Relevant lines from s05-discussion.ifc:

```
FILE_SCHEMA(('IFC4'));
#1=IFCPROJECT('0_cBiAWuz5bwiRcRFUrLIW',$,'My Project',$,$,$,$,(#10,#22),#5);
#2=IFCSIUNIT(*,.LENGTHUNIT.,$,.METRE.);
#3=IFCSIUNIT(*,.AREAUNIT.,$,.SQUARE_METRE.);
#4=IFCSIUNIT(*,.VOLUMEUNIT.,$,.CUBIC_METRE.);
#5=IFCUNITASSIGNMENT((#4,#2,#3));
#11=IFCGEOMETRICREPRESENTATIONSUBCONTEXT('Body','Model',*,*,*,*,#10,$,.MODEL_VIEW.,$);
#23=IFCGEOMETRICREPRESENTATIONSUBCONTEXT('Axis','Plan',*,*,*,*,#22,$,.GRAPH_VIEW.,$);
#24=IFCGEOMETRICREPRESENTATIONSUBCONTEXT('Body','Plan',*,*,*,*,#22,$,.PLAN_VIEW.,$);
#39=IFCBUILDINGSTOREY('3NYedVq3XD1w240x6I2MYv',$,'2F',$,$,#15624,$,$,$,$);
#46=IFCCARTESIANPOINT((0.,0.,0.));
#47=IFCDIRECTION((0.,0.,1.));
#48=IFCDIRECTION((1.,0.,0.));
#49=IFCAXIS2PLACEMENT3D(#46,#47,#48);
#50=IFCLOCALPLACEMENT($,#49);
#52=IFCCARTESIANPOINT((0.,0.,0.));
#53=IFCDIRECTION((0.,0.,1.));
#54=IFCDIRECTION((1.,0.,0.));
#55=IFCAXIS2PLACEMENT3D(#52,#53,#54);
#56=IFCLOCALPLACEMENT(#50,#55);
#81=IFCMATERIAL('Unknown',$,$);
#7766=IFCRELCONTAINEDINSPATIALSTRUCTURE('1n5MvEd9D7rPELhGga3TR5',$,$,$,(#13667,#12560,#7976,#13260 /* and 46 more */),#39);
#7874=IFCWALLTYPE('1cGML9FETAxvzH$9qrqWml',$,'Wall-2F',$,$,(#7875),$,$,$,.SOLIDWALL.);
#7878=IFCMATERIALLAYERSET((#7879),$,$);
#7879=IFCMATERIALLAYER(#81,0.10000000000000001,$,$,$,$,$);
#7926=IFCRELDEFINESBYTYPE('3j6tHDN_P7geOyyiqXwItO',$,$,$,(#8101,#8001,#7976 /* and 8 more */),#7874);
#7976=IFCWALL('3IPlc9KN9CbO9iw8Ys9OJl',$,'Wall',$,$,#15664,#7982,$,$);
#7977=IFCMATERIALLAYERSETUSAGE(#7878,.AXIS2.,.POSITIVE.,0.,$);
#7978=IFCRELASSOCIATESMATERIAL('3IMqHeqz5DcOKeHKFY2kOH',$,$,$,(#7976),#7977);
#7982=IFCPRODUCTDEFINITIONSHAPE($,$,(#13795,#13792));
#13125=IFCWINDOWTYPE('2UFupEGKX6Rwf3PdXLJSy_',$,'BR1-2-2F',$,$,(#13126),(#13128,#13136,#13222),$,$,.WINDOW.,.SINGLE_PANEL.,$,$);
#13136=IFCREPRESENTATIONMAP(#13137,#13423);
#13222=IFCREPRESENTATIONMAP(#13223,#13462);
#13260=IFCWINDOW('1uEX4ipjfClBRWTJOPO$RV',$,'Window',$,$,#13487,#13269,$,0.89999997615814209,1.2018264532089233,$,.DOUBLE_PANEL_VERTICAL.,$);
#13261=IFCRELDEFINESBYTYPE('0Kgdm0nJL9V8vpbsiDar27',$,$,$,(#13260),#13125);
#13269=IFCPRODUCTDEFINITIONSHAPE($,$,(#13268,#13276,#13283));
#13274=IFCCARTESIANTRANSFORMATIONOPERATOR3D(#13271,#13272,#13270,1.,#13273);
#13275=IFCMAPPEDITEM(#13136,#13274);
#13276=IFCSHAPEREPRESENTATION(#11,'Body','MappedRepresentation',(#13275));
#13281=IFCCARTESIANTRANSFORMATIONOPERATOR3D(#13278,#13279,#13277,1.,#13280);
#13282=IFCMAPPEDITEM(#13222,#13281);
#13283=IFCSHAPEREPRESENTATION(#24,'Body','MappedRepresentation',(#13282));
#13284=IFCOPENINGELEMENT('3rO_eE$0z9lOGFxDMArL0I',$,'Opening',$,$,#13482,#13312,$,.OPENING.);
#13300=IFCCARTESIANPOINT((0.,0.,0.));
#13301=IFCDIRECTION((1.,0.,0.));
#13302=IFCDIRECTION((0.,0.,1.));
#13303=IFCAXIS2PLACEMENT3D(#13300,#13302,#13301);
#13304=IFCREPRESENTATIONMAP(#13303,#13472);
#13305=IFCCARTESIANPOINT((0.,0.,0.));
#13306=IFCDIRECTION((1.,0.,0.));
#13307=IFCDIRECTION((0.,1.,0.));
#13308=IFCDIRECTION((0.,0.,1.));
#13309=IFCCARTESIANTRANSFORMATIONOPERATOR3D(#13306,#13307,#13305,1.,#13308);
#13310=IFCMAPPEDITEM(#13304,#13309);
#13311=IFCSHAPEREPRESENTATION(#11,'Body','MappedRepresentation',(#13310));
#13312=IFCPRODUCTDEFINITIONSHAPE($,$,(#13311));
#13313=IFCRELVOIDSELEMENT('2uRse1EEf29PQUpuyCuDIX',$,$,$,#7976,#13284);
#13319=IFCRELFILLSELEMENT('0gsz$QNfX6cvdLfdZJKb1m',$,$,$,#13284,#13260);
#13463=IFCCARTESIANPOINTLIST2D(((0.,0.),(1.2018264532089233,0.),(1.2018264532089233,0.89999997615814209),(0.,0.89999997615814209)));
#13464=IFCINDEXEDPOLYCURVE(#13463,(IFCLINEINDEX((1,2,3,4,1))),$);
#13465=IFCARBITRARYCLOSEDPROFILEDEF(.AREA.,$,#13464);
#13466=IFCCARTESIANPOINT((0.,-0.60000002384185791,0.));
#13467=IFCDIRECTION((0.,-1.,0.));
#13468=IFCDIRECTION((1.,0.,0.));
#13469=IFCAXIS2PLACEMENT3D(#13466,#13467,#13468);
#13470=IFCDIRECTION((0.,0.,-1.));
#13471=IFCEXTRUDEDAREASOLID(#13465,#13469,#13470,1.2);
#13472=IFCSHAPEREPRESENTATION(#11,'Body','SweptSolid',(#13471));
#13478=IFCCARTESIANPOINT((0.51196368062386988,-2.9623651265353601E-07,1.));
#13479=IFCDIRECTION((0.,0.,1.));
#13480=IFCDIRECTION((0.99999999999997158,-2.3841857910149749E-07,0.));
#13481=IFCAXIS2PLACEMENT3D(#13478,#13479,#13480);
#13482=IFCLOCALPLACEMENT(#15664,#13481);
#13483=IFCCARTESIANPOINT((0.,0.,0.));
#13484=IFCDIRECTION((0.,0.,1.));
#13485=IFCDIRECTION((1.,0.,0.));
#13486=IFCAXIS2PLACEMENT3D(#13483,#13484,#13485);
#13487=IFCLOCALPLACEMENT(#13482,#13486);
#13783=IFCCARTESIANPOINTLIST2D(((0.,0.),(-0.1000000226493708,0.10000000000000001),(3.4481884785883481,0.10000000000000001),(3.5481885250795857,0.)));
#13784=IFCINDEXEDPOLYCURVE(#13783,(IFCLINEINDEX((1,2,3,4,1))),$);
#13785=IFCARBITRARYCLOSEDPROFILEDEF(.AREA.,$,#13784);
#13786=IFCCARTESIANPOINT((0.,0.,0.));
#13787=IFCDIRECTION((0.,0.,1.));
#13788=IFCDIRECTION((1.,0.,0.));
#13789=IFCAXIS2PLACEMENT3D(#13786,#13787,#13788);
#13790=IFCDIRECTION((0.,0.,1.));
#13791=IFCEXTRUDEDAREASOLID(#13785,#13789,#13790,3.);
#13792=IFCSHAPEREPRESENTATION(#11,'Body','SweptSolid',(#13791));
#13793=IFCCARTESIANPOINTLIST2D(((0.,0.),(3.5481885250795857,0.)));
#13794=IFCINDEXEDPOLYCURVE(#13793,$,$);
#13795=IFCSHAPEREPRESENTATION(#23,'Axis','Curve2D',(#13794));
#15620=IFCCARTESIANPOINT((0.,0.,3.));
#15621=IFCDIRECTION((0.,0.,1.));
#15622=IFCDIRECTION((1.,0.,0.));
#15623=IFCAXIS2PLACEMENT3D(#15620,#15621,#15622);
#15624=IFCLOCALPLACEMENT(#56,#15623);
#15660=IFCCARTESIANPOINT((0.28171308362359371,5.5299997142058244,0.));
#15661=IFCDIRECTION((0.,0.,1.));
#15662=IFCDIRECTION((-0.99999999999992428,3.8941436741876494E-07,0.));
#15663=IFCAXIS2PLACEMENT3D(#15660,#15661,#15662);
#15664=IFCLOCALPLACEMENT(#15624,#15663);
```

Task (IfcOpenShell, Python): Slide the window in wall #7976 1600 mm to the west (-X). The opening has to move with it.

```python
import ifcopenshell
import ifcopenshell.api.geometry
import ifcopenshell.util.placement
import ifcopenshell.util.unit

model = ifcopenshell.open("s05-discussion.ifc")
unit_scale = ifcopenshell.util.unit.calculate_unit_scale(model)

window = model.by_guid("1uEX4ipjfClBRWTJOPO$RV")
opening = window.FillsVoids[0].RelatingOpeningElement
wall = opening.VoidsElements[0].RelatingBuildingElement

wall_matrix = ifcopenshell.util.placement.get_local_placement(wall.ObjectPlacement)
shift = wall_matrix[:3, 0] * 1.6 / unit_scale
before = ifcopenshell.util.placement.get_local_placement(window.ObjectPlacement)[:3, 3].copy()

# The window is placed relative to its opening, so it follows when the opening moves.
matrix = ifcopenshell.util.placement.get_local_placement(opening.ObjectPlacement)
matrix[:3, 3] += shift
ifcopenshell.api.geometry.edit_object_placement(
    model, product=opening, matrix=matrix, is_si=False, should_transform_children=True
)

after = ifcopenshell.util.placement.get_local_placement(window.ObjectPlacement)[:3, 3]
print("window moved by", (after - before).round(3) + 0.0)

model.write("s05-discussion-out.ifc")
```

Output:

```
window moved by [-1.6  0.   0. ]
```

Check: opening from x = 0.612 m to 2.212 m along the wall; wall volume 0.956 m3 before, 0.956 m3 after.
